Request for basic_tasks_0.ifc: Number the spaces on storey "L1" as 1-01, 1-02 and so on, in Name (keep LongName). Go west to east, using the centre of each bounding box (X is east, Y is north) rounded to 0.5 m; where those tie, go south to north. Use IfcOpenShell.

First a look at what the model holds.

```python
import ifcopenshell
import ifcopenshell.util.element
import ifcopenshell.util.placement

model = ifcopenshell.open("basic_tasks_0.ifc")
print(model.schema)
storey = next(s for s in model.by_type("IfcBuildingStorey") if s.Name == "L1")
spaces = [e for e in ifcopenshell.util.element.get_decomposition(storey) if e.is_a("IfcSpace")]
for e in sorted(spaces, key=lambda e: e.id()):
    origin = ifcopenshell.util.placement.get_local_placement(e.ObjectPlacement)[:3, 3]
    print(e.id(), e.Name, e.LongName, origin.round(2) + 0.0, sep=" | ")
```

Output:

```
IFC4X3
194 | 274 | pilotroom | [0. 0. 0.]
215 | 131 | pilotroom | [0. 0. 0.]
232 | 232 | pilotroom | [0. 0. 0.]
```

```python
import ifcopenshell
import ifcopenshell.geom
import ifcopenshell.util.element
import ifcopenshell.util.shape

model = ifcopenshell.open("basic_tasks_0.ifc")
settings = ifcopenshell.geom.settings()
settings.set("use-world-coords", True)


def centre(element):
    shape = ifcopenshell.geom.create_shape(settings, element)
    return ifcopenshell.util.shape.get_bbox_centroid(shape.geometry)


storey = next(s for s in model.by_type("IfcBuildingStorey") if s.Name == "L1")
spaces = [e for e in ifcopenshell.util.element.get_decomposition(storey) if e.is_a("IfcSpace")]

# Insertion points can sit at a corner or the storey origin, so sort by the geometry (in metres).
centres = {e: centre(e) for e in spaces}
spaces.sort(key=lambda e: (round(centres[e][0] / 0.5), centres[e][1]))

for i, e in enumerate(spaces, start=1):
    number = f"1-{i:02d}"
    e.Name = number
    print(e.id(), number)

model.write("basic_tasks_0_rev.ifc")
```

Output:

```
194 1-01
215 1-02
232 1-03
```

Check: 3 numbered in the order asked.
